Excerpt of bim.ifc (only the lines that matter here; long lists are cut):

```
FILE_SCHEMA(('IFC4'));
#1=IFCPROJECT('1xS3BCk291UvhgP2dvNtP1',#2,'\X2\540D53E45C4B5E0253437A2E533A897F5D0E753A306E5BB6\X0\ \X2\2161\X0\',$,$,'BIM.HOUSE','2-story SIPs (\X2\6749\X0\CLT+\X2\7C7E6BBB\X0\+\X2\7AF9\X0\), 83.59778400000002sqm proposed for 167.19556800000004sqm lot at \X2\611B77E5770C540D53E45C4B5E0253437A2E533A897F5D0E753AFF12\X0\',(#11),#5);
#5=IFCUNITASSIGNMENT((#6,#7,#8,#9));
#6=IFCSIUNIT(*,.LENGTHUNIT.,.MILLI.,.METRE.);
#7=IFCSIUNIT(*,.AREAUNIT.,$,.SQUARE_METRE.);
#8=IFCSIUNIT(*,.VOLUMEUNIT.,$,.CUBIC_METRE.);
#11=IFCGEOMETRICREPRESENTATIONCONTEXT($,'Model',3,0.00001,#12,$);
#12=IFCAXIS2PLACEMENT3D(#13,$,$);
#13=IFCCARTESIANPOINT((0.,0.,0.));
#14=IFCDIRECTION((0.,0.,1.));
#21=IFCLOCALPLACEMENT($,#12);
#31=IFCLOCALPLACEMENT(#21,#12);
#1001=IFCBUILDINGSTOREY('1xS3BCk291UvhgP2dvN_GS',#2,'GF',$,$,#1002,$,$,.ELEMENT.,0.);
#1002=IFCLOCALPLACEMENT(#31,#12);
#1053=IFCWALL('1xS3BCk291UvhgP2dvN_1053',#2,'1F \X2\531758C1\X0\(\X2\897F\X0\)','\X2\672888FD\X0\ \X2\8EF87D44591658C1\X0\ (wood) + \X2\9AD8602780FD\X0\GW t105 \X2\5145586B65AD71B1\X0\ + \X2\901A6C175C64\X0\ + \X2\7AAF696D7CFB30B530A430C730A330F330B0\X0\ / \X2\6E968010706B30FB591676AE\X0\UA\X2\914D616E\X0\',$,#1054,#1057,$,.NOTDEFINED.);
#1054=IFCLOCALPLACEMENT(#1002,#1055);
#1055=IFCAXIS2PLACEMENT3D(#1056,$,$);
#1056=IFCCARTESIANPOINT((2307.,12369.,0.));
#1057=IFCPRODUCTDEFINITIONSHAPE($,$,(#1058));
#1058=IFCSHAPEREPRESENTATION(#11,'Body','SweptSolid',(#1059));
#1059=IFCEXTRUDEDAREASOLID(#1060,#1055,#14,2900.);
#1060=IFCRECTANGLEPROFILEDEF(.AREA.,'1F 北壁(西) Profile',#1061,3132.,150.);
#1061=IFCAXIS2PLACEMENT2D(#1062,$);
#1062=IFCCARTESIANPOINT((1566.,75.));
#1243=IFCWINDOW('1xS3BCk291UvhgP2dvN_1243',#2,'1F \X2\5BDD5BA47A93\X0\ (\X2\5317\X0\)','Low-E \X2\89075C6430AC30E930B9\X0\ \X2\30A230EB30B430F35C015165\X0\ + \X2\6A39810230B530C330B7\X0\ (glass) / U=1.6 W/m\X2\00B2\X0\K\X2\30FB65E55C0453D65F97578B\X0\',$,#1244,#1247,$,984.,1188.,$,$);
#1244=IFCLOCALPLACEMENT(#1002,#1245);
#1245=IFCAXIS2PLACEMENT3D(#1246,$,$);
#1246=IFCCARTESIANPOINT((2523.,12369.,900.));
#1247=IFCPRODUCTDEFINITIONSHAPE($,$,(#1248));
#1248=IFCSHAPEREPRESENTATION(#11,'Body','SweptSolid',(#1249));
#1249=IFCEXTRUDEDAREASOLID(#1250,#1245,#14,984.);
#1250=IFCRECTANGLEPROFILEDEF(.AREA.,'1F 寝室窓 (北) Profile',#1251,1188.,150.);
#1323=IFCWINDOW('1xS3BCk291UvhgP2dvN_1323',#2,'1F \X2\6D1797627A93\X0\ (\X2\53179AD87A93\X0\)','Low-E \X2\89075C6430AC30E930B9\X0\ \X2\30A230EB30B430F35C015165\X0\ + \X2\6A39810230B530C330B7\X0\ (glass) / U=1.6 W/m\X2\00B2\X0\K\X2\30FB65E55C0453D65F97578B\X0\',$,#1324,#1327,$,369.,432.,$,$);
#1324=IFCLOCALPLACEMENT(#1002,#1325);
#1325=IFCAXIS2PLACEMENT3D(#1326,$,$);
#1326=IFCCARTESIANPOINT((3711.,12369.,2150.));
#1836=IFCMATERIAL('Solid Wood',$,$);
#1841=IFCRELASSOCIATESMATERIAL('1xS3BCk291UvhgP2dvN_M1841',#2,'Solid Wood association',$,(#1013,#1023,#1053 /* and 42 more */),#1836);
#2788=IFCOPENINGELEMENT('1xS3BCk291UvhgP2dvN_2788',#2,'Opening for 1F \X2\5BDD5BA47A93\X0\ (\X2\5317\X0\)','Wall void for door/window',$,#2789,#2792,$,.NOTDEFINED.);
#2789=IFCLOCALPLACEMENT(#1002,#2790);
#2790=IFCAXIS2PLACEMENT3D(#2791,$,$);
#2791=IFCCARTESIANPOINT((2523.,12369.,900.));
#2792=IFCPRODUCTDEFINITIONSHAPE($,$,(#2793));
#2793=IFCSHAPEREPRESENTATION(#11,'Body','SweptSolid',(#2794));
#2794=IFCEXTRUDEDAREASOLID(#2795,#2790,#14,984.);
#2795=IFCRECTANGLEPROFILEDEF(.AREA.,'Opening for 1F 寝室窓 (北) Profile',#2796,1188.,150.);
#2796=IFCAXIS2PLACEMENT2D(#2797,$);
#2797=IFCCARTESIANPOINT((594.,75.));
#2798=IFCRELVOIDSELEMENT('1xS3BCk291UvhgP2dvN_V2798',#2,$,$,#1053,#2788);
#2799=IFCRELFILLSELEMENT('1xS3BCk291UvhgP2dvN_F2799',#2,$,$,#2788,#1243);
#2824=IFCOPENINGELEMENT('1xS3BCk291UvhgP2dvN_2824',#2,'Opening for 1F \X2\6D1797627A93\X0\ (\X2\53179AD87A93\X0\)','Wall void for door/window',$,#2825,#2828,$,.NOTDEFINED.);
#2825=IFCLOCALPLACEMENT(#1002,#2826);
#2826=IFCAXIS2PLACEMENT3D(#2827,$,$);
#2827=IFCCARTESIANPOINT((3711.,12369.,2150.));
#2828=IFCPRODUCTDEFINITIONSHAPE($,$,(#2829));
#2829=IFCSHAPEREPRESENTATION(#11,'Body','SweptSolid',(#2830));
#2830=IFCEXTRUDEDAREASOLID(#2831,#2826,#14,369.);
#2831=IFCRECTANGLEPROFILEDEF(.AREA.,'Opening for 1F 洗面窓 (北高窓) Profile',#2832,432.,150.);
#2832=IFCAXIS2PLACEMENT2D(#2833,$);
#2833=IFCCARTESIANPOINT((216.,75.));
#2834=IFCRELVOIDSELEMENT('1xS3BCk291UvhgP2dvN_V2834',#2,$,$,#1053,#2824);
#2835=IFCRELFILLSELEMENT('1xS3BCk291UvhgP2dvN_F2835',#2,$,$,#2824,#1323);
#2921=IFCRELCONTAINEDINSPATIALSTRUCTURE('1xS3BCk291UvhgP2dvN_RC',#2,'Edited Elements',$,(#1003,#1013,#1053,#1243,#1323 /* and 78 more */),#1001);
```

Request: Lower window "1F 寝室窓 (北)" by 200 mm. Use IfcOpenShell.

```python
import numpy as np
import ifcopenshell
import ifcopenshell.api.geometry
import ifcopenshell.util.placement
import ifcopenshell.util.unit

model = ifcopenshell.open("bim.ifc")
unit_scale = ifcopenshell.util.unit.calculate_unit_scale(model)

window = model.by_guid("1xS3BCk291UvhgP2dvN_1243")
opening = window.FillsVoids[0].RelatingOpeningElement
dz = -0.2 / unit_scale

shift = np.array([0.0, 0.0, dz])
# The window is not placed relative to its opening, so move both.
for product in (opening, window):
    matrix = ifcopenshell.util.placement.get_local_placement(product.ObjectPlacement)
    matrix[:3, 3] += shift
    ifcopenshell.api.geometry.edit_object_placement(model, product=product, matrix=matrix, is_si=False)

print(f"moved by {dz * unit_scale:+.3f} m")

model.write("bim_v2.ifc")
```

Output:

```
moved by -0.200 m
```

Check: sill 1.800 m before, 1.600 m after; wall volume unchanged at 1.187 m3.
